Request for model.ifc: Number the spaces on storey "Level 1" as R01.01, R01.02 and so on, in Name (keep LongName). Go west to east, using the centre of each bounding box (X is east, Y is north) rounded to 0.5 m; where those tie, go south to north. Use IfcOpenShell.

First a look at what the model holds.

```python
import ifcopenshell
import ifcopenshell.util.element
import ifcopenshell.util.placement

model = ifcopenshell.open("model.ifc")
print(model.schema)
storey = next(s for s in model.by_type("IfcBuildingStorey") if s.Name == "Level 1")
spaces = [e for e in ifcopenshell.util.element.get_decomposition(storey) if e.is_a("IfcSpace")]
for e in sorted(spaces, key=lambda e: e.id()):
    origin = ifcopenshell.util.placement.get_local_placement(e.ObjectPlacement)[:3, 3]
    print(e.id(), e.Name, e.LongName, origin.round(2) + 0.0, sep=" | ")
```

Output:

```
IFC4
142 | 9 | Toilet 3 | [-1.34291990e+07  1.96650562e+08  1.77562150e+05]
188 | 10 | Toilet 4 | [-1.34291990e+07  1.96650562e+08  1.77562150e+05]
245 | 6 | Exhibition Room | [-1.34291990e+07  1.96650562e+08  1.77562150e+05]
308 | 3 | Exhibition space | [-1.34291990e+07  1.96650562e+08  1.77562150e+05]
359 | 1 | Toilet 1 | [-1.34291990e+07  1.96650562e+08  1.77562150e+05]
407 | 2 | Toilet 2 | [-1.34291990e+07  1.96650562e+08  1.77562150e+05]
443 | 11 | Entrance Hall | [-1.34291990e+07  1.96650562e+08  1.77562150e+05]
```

```python
import ifcopenshell
import ifcopenshell.geom
import ifcopenshell.util.element
import ifcopenshell.util.shape

model = ifcopenshell.open("model.ifc")
settings = ifcopenshell.geom.settings()
settings.set("use-world-coords", True)


def centre(element):
    shape = ifcopenshell.geom.create_shape(settings, element)
    return ifcopenshell.util.shape.get_bbox_centroid(shape.geometry)


storey = next(s for s in model.by_type("IfcBuildingStorey") if s.Name == "Level 1")
spaces = [e for e in ifcopenshell.util.element.get_decomposition(storey) if e.is_a("IfcSpace")]

# Insertion points can sit at a corner or the storey origin, so sort by the geometry (in metres).
centres = {e: centre(e) for e in spaces}
spaces.sort(key=lambda e: (round(centres[e][0] / 0.5), centres[e][1]))

for i, e in enumerate(spaces, start=1):
    number = f"R01.{i:02d}"
    e.Name = number
    print(e.id(), number)

model.write("model_rev.ifc")
```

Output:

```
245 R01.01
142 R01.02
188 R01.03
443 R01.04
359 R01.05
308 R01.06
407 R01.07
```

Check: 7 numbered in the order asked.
